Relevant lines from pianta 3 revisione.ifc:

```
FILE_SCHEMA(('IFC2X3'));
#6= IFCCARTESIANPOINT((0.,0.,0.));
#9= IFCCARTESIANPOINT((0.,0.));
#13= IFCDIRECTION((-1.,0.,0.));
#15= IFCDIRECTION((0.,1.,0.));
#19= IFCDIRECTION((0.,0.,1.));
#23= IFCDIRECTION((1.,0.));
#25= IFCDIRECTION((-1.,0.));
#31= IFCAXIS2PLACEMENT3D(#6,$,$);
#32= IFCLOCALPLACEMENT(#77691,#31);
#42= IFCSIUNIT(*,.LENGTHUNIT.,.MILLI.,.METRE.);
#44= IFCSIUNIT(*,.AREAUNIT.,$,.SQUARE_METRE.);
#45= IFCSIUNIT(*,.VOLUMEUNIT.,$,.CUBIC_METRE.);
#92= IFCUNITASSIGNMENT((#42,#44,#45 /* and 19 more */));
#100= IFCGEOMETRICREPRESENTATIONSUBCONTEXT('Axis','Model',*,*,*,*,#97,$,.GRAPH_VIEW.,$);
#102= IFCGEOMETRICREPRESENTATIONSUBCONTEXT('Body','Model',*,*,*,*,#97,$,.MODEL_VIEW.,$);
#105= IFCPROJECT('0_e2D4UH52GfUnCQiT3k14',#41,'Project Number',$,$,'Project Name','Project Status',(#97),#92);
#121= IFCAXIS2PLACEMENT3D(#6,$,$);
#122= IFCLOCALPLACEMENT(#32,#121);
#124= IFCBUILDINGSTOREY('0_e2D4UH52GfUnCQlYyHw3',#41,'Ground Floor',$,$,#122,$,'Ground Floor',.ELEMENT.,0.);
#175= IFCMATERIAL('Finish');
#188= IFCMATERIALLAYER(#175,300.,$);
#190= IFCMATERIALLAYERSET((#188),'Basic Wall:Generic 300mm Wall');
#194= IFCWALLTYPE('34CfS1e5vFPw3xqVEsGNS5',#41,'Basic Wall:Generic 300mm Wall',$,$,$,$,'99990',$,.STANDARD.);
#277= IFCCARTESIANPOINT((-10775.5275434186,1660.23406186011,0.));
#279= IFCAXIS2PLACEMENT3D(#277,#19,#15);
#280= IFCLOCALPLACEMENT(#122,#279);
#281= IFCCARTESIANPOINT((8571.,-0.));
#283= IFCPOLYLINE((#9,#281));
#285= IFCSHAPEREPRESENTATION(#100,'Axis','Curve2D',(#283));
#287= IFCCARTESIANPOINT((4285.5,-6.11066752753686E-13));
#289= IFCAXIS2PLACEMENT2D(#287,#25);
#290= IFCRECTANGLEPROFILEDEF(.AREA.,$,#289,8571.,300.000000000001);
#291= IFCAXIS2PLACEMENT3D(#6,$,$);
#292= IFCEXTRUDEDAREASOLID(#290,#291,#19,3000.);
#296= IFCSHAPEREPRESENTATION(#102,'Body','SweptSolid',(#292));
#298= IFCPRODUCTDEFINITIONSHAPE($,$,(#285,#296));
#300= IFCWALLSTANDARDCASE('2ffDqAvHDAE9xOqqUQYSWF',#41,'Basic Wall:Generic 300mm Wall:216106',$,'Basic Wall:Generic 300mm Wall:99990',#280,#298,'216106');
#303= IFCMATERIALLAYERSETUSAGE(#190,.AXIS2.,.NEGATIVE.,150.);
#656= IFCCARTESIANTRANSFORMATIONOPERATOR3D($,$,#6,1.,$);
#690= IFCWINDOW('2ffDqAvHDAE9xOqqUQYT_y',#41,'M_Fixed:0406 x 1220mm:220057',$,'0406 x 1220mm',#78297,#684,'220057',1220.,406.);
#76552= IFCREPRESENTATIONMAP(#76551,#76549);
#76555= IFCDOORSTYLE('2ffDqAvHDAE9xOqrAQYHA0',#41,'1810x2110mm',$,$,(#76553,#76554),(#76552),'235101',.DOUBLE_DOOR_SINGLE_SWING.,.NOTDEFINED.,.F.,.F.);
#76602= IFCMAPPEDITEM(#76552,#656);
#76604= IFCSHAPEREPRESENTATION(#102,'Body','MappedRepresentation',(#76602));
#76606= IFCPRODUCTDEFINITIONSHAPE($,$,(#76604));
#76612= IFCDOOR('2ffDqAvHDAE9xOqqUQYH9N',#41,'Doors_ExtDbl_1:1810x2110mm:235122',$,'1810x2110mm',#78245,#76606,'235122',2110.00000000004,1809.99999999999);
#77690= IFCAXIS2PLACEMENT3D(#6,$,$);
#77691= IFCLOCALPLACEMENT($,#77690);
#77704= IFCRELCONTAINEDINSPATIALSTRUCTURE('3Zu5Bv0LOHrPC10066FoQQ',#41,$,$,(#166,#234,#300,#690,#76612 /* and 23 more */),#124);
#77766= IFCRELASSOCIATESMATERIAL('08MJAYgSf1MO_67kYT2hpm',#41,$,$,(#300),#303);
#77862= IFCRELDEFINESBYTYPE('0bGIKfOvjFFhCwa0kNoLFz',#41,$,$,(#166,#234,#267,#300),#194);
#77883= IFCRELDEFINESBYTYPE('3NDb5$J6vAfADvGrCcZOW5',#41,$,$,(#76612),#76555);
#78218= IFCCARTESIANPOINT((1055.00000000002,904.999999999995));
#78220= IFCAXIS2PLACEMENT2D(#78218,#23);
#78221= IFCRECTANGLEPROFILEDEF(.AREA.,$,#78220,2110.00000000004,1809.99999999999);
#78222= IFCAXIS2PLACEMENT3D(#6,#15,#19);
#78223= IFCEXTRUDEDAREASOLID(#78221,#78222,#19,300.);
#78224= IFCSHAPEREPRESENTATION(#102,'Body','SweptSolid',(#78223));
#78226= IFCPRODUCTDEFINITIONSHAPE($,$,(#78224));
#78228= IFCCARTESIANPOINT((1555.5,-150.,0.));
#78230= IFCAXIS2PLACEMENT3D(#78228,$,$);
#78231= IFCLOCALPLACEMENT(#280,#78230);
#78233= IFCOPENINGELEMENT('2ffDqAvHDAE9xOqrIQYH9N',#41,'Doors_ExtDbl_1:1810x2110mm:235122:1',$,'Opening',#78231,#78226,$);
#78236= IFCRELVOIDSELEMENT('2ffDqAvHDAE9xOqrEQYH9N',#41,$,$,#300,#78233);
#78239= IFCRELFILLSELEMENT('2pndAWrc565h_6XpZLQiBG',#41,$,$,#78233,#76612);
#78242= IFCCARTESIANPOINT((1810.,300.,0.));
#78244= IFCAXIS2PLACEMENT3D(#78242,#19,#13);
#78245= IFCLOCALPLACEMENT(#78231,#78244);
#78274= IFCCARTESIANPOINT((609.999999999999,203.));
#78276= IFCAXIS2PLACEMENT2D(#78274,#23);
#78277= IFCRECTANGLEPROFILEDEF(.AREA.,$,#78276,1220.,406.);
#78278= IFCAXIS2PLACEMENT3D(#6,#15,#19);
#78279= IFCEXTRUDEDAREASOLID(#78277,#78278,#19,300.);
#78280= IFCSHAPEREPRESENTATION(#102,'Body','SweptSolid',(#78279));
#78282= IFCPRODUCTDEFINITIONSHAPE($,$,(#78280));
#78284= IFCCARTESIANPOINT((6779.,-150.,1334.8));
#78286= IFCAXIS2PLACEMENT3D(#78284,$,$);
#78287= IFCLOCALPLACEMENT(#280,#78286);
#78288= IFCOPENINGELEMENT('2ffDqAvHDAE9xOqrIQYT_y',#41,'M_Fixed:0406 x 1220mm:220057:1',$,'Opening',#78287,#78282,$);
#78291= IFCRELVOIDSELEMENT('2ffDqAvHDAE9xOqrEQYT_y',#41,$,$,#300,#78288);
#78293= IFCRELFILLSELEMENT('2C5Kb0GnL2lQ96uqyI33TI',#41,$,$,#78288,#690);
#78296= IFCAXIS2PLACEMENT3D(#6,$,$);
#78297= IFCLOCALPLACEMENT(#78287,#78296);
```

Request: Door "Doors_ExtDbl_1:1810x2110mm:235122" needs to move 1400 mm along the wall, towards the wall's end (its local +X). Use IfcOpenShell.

```python
import ifcopenshell
import ifcopenshell.api.geometry
import ifcopenshell.util.placement
import ifcopenshell.util.unit

model = ifcopenshell.open("pianta 3 revisione.ifc")
unit_scale = ifcopenshell.util.unit.calculate_unit_scale(model)

door = model.by_id(76612)
opening = door.FillsVoids[0].RelatingOpeningElement
wall = opening.VoidsElements[0].RelatingBuildingElement

wall_matrix = ifcopenshell.util.placement.get_local_placement(wall.ObjectPlacement)
shift = wall_matrix[:3, 0] * 1.4 / unit_scale
before = ifcopenshell.util.placement.get_local_placement(door.ObjectPlacement)[:3, 3].copy()

# The door is placed relative to its opening, so it follows when the opening moves.
matrix = ifcopenshell.util.placement.get_local_placement(opening.ObjectPlacement)
matrix[:3, 3] += shift
ifcopenshell.api.geometry.edit_object_placement(
    model, product=opening, matrix=matrix, is_si=False, should_transform_children=True
)

after = ifcopenshell.util.placement.get_local_placement(door.ObjectPlacement)[:3, 3]
print("door moved by", (after - before).round(3) + 0.0)

model.write("pianta 3 revisione_updated.ifc")
```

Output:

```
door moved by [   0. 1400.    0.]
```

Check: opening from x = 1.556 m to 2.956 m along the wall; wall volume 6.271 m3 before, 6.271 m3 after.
